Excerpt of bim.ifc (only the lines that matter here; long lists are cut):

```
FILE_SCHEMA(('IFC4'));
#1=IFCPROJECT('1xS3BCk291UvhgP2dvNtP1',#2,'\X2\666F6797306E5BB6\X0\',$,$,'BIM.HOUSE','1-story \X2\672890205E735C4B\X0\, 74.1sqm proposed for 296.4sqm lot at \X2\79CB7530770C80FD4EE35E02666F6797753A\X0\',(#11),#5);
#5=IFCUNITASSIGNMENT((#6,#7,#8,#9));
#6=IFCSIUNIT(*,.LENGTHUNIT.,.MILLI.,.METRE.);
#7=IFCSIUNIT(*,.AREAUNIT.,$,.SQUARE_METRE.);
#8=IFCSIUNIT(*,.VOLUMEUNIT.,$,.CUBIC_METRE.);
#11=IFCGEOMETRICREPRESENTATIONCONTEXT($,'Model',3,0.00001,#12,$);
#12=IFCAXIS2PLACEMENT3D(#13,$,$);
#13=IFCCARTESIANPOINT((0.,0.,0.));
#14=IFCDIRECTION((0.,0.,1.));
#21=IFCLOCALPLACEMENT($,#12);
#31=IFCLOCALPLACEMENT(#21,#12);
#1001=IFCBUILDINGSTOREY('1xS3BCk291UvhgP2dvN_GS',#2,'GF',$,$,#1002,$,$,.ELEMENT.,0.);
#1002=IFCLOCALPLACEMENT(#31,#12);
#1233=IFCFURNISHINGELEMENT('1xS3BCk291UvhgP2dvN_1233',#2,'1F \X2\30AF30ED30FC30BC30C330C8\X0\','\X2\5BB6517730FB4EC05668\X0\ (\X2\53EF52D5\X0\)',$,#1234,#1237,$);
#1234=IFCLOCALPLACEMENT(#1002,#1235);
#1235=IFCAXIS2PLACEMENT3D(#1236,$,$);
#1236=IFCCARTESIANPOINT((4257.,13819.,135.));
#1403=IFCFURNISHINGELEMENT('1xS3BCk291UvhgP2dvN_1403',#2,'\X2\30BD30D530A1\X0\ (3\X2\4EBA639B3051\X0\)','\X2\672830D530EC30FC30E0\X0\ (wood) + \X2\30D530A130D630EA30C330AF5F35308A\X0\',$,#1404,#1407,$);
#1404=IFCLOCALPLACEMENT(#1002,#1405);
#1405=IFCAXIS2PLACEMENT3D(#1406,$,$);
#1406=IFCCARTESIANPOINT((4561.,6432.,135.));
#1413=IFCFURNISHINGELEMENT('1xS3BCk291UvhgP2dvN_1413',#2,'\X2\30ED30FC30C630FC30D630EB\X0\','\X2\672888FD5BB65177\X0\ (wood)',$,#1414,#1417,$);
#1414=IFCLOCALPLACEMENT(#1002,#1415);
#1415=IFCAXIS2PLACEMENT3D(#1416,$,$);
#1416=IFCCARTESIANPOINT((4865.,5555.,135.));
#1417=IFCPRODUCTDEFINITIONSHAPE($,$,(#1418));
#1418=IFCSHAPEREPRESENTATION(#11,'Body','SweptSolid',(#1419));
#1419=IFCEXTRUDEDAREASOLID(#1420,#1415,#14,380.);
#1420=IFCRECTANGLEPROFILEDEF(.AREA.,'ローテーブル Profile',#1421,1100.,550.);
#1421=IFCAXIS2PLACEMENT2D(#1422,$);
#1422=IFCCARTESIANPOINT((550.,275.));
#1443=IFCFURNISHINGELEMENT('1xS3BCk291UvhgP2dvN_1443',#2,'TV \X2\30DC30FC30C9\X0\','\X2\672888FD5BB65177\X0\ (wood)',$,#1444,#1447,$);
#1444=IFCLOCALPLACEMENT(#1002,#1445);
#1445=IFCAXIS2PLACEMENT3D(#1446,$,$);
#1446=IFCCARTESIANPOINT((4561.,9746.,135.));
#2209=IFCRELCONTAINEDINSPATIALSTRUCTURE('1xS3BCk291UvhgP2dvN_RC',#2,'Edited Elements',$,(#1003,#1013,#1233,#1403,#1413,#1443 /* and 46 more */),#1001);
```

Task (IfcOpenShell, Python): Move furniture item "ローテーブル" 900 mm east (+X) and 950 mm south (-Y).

```python
import ifcopenshell
import ifcopenshell.api.geometry
import ifcopenshell.util.placement

model = ifcopenshell.open("bim.ifc")

item = model.by_guid("1xS3BCk291UvhgP2dvN_1413")
matrix = ifcopenshell.util.placement.get_local_placement(item.ObjectPlacement)
matrix[0, 3] += 900.0
matrix[1, 3] -= 950.0
ifcopenshell.api.geometry.edit_object_placement(model, product=item, matrix=matrix, is_si=False)

print(ifcopenshell.util.placement.get_local_placement(item.ObjectPlacement).round(3) + 0.0)

model.write("bim_updated.ifc")
```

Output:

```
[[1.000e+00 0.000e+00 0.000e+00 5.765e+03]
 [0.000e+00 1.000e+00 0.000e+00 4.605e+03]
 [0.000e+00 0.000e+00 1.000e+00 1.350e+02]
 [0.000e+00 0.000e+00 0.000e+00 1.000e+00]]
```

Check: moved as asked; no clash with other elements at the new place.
